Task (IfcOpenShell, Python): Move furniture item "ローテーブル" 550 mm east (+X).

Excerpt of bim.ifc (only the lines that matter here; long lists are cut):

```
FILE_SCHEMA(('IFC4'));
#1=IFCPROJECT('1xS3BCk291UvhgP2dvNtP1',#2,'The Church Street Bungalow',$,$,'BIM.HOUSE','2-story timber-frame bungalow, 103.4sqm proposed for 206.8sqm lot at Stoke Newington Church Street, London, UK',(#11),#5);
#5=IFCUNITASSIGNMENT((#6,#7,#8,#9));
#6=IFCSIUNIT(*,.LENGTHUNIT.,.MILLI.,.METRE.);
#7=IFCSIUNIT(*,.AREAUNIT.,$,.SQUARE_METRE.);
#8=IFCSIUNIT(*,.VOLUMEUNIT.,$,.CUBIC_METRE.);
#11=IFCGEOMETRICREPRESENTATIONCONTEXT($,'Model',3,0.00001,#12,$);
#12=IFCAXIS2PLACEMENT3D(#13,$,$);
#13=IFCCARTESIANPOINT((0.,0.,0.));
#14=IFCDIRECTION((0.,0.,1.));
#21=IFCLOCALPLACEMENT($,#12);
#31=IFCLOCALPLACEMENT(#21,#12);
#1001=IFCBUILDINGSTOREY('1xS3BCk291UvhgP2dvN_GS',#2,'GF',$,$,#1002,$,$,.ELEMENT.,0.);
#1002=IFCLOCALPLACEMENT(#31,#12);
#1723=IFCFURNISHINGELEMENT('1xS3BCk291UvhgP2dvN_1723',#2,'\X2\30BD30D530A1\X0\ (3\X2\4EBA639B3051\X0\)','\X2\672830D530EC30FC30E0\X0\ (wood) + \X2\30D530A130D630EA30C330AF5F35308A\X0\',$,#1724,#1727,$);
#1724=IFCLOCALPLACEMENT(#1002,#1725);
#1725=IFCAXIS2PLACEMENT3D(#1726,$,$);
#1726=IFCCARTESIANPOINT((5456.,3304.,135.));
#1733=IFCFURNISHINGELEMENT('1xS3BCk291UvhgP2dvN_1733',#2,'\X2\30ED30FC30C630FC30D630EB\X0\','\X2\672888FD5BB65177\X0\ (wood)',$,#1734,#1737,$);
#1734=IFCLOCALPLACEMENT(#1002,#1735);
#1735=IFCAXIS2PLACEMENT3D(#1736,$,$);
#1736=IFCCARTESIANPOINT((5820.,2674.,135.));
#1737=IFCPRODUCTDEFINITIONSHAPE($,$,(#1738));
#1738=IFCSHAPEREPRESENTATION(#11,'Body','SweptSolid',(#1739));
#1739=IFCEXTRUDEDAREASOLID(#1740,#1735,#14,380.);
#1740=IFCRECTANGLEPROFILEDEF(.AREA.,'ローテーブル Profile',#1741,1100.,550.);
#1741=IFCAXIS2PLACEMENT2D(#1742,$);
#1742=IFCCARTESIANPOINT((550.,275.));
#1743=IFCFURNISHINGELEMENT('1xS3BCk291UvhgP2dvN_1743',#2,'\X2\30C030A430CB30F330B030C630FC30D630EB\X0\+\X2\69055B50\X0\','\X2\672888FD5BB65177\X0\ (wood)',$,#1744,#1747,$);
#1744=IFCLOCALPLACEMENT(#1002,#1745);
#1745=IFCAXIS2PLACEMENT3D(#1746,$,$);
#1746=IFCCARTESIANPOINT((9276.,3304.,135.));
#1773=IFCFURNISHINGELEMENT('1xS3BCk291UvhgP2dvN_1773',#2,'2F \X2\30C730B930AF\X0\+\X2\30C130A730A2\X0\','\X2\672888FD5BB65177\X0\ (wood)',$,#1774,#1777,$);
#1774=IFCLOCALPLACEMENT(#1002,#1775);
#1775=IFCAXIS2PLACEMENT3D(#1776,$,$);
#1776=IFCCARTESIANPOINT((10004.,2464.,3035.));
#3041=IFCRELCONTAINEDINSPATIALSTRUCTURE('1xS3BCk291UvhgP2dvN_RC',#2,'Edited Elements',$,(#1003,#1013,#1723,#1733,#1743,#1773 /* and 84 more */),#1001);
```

```python
import ifcopenshell
import ifcopenshell.api.geometry
import ifcopenshell.util.placement

model = ifcopenshell.open("bim.ifc")

item = model.by_guid("1xS3BCk291UvhgP2dvN_1733")
matrix = ifcopenshell.util.placement.get_local_placement(item.ObjectPlacement)
matrix[0, 3] += 550.0
ifcopenshell.api.geometry.edit_object_placement(model, product=item, matrix=matrix, is_si=False)

print(ifcopenshell.util.placement.get_local_placement(item.ObjectPlacement).round(3) + 0.0)

model.write("bim_v2.ifc")
```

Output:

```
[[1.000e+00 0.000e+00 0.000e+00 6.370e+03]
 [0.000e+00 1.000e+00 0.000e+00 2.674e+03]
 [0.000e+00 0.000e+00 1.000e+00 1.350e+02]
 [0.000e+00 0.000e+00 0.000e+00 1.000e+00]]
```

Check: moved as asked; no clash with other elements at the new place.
